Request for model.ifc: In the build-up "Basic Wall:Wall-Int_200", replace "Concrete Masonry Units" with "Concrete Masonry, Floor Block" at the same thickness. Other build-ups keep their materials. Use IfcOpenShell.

First a look at what the model holds.

```python
import ifcopenshell
import ifcopenshell.util.element

model = ifcopenshell.open("model.ifc")
print(model.schema)
for layer_set in model.by_type("IfcMaterialLayerSet"):
    if layer_set.LayerSetName == "Basic Wall:Wall-Int_200":
        for layer in layer_set.MaterialLayers:
            print(layer.id(), layer.Material and layer.Material.Name, layer.LayerThickness, sep=" | ")
        print(len(ifcopenshell.util.element.get_elements_by_material(model, layer_set)), "elements and types use it")
print(sorted(m.Name for m in model.by_type("IfcMaterial") if m.Name)[:60])
```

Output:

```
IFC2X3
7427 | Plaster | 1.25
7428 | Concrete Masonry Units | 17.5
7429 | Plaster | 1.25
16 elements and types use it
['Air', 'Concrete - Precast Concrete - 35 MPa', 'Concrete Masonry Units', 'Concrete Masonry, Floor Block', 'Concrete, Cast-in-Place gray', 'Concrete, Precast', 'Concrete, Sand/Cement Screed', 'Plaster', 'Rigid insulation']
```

```python
import ifcopenshell
import ifcopenshell.api.material

model = ifcopenshell.open("model.ifc")

layer_set = next(s for s in model.by_type("IfcMaterialLayerSet") if s.LayerSetName == "Basic Wall:Wall-Int_200")
layer = next(l for l in layer_set.MaterialLayers if l.Material and l.Material.Name == "Concrete Masonry Units")
material = next(m for m in model.by_type("IfcMaterial") if m.Name == "Concrete Masonry, Floor Block")

# Point this one layer at the other material; renaming the old one would change it everywhere.
ifcopenshell.api.material.edit_layer(model, layer=layer, attributes={}, material=material)

print([l.Material.Name if l.Material else None for l in layer_set.MaterialLayers])

model.write("model_v2.ifc")
```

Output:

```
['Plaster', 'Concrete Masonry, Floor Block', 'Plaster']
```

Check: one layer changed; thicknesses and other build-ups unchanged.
